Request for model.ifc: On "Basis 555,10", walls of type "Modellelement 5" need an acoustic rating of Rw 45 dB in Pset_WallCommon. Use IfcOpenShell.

First a look at what the model holds.

```python
import ifcopenshell
import ifcopenshell.util.element

model = ifcopenshell.open("model.ifc")
print(model.schema)
storey = next(s for s in model.by_type("IfcBuildingStorey") if s.Name == "Basis 555,10")
walls = [e for e in ifcopenshell.util.element.get_decomposition(storey) if e.is_a("IfcWall")]
seen = {}
for e in walls:
    element_type = ifcopenshell.util.element.get_type(e)
    key = (element_type.Name if element_type != e and element_type else None, ifcopenshell.util.element.get_pset(e, "Pset_WallCommon", "AcousticRating"))
    seen[key] = seen.get(key, 0) + 1
for (name, value), count in sorted(seen.items(), key=str):
    print(count, "x", name, "|", value)
```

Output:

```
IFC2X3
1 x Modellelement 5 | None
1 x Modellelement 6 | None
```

```python
import ifcopenshell
import ifcopenshell.api.pset
import ifcopenshell.util.element

model = ifcopenshell.open("model.ifc")

storey = next(s for s in model.by_type("IfcBuildingStorey") if s.Name == "Basis 555,10")
walls = [e for e in ifcopenshell.util.element.get_decomposition(storey) if e.is_a("IfcWall")]

count = 0
for e in walls:
    element_type = ifcopenshell.util.element.get_type(e)
    if element_type in (None, e) or element_type.Name != "Modellelement 5":
        continue
    # add_pset returns the element's existing set when there is one.
    pset = ifcopenshell.api.pset.add_pset(model, product=e, name="Pset_WallCommon")
    ifcopenshell.api.pset.edit_pset(model, pset=pset, properties={"AcousticRating": "Rw 45 dB"})
    count += 1

print(count, "walls updated")

model.write("model_updated.ifc")
```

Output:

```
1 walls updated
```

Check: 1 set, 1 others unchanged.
